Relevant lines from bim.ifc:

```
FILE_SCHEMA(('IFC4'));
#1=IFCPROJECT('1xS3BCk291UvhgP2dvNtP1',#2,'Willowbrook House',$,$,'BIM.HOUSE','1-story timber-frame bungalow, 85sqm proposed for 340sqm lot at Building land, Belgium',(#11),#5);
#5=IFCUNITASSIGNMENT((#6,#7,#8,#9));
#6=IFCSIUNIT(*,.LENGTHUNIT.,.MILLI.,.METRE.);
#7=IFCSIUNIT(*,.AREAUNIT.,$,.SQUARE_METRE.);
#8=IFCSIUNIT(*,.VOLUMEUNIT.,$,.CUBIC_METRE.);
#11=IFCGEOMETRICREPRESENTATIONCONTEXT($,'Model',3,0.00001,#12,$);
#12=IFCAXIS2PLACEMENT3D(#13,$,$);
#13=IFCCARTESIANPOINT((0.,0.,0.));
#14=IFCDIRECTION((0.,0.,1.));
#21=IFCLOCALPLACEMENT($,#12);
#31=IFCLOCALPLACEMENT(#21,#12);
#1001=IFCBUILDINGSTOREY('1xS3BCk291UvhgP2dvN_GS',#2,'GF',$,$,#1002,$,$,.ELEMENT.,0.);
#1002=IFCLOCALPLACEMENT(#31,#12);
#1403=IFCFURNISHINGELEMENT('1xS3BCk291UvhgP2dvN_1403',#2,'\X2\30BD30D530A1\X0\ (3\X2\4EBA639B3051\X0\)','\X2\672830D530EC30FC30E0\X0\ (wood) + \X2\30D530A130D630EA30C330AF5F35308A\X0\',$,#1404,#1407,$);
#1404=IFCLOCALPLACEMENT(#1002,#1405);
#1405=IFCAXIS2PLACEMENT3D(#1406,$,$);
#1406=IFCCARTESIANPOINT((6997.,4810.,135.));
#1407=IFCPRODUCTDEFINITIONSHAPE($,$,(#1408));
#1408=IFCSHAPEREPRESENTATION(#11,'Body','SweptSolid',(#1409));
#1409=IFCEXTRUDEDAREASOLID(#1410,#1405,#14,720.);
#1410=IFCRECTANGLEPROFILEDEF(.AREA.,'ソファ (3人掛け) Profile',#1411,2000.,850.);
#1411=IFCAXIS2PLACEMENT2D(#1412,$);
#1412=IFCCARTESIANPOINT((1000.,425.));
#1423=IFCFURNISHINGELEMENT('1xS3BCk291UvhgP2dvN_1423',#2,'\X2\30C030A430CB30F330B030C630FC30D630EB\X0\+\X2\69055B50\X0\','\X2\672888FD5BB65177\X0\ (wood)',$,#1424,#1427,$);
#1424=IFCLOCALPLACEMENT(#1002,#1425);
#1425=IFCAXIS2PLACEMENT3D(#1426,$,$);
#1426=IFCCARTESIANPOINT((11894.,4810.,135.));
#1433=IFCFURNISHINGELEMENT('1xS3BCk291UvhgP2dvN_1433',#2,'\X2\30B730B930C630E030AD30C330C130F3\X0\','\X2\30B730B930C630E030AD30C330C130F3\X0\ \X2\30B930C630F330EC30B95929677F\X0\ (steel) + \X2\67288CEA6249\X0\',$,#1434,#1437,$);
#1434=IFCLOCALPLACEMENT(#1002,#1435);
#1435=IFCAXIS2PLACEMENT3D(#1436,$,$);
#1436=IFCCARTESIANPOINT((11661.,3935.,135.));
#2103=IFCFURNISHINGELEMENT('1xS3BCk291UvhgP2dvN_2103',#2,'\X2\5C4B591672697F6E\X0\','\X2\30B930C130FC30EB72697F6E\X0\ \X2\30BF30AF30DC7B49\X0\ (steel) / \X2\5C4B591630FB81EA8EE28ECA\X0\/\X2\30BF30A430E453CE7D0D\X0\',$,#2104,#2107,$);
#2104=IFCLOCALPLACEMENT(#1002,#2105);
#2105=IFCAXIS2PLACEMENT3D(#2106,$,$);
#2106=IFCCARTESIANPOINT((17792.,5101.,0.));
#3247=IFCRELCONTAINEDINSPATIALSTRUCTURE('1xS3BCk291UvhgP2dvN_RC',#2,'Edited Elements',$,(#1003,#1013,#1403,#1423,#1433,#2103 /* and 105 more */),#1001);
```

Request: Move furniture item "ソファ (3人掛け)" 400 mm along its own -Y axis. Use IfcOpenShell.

```python
import ifcopenshell
import ifcopenshell.api.geometry
import ifcopenshell.util.placement
import ifcopenshell.util.unit

model = ifcopenshell.open("bim.ifc")
unit_scale = ifcopenshell.util.unit.calculate_unit_scale(model)

item = model.by_guid("1xS3BCk291UvhgP2dvN_1403")
matrix = ifcopenshell.util.placement.get_local_placement(item.ObjectPlacement)
matrix[:3, 3] -= matrix[:3, 1] * 0.4 / unit_scale
ifcopenshell.api.geometry.edit_object_placement(model, product=item, matrix=matrix, is_si=False)

print(ifcopenshell.util.placement.get_local_placement(item.ObjectPlacement).round(3) + 0.0)

model.write("bim_edited.ifc")
```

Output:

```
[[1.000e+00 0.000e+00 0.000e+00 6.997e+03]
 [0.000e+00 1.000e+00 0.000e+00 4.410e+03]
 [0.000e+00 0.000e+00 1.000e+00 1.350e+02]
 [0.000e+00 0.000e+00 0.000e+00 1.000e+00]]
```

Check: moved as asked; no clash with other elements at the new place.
